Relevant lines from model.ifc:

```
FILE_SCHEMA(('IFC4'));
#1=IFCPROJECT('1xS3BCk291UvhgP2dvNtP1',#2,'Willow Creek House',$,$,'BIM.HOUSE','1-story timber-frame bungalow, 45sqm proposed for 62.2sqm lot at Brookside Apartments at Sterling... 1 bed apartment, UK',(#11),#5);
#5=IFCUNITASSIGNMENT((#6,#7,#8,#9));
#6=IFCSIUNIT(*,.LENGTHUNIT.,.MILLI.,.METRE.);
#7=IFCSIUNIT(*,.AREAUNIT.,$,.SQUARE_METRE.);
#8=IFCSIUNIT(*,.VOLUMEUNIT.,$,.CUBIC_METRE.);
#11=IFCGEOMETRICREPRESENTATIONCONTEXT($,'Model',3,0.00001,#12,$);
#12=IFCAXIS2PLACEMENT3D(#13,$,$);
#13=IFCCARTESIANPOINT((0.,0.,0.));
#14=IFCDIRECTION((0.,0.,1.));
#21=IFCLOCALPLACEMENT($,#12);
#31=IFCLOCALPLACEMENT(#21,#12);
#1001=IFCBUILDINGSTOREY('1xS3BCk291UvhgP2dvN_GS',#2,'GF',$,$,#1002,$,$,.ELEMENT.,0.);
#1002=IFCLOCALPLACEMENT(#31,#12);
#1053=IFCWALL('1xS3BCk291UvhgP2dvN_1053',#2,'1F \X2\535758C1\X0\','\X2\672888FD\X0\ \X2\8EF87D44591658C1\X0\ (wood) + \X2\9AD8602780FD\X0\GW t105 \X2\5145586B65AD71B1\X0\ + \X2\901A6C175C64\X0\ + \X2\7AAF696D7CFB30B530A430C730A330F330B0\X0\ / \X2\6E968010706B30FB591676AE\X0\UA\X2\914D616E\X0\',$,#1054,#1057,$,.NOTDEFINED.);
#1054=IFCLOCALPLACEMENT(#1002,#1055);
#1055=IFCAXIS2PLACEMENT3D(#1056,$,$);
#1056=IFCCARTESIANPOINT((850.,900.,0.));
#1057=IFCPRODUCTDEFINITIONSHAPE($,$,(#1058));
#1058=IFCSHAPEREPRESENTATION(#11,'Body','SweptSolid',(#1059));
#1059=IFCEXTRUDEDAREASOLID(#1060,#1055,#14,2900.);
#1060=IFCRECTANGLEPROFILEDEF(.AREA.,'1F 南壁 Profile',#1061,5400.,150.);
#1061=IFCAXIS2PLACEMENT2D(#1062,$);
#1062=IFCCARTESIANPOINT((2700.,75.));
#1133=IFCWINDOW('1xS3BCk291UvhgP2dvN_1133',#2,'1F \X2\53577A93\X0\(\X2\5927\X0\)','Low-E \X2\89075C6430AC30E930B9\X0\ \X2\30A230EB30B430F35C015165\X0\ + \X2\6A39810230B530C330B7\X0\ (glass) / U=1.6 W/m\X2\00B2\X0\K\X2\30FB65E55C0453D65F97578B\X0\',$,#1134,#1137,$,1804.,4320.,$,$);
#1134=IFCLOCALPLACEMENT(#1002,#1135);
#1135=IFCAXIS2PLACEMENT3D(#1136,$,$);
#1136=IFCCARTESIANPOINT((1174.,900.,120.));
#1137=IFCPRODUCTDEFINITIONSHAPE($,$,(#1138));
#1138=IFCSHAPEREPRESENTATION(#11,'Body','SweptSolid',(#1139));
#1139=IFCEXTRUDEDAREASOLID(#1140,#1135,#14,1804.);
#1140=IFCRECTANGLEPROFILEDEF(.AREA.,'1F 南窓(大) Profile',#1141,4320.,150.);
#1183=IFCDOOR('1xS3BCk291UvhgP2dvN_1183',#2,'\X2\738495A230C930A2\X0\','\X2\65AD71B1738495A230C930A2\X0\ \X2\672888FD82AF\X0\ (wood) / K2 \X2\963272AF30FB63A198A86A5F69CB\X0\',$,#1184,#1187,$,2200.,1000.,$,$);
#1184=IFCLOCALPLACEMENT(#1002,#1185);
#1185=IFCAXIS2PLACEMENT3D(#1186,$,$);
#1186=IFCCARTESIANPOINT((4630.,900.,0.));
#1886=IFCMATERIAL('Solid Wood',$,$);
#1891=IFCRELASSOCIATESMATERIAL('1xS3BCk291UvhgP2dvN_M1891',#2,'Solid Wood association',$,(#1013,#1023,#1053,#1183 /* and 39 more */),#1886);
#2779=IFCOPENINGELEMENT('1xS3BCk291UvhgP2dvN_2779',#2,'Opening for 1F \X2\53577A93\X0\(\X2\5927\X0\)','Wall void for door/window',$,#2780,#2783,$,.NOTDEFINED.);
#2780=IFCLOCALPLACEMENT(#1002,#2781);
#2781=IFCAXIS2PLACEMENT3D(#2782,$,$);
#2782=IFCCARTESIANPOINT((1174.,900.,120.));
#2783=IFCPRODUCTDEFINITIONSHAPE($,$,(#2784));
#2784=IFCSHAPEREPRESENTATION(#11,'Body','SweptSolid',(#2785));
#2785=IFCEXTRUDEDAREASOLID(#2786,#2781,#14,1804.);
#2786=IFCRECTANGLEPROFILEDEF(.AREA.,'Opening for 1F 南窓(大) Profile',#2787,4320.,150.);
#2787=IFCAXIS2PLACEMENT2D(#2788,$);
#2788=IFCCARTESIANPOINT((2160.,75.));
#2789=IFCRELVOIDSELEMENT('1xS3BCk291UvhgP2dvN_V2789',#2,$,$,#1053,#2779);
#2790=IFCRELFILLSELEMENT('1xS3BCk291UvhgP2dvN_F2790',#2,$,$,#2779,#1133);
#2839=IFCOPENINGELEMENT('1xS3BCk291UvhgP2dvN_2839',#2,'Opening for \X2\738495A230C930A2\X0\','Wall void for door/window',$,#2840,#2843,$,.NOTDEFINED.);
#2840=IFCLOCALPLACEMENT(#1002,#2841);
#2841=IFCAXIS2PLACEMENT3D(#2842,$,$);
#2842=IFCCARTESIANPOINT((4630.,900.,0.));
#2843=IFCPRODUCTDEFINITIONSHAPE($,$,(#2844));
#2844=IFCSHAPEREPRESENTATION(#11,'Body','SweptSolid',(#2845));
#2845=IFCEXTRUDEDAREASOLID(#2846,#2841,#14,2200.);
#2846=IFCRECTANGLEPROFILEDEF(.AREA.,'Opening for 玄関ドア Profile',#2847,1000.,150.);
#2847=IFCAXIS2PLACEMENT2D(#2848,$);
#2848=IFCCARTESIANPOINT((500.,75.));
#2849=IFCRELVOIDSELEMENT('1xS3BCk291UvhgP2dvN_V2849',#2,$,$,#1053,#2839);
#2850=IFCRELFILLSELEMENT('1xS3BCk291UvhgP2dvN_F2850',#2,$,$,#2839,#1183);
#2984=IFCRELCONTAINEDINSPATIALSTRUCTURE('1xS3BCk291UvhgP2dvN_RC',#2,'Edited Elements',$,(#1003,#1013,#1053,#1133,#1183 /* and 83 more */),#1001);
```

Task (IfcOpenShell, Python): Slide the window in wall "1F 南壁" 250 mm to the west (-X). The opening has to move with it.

```python
import ifcopenshell
import ifcopenshell.api.geometry
import ifcopenshell.util.placement
import ifcopenshell.util.unit

model = ifcopenshell.open("model.ifc")
unit_scale = ifcopenshell.util.unit.calculate_unit_scale(model)

window = model.by_guid("1xS3BCk291UvhgP2dvN_1133")
opening = window.FillsVoids[0].RelatingOpeningElement
wall = opening.VoidsElements[0].RelatingBuildingElement

wall_matrix = ifcopenshell.util.placement.get_local_placement(wall.ObjectPlacement)
shift = wall_matrix[:3, 0] * -0.25 / unit_scale
before = ifcopenshell.util.placement.get_local_placement(window.ObjectPlacement)[:3, 3].copy()

# The window is not placed relative to its opening, so move both.
for product in (opening, window):
    matrix = ifcopenshell.util.placement.get_local_placement(product.ObjectPlacement)
    matrix[:3, 3] += shift
    ifcopenshell.api.geometry.edit_object_placement(model, product=product, matrix=matrix, is_si=False)

after = ifcopenshell.util.placement.get_local_placement(window.ObjectPlacement)[:3, 3]
print("window moved by", (after - before).round(3) + 0.0)

model.write("model_rev.ifc")
```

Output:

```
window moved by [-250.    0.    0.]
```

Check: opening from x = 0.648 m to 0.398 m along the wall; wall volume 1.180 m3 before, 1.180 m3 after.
